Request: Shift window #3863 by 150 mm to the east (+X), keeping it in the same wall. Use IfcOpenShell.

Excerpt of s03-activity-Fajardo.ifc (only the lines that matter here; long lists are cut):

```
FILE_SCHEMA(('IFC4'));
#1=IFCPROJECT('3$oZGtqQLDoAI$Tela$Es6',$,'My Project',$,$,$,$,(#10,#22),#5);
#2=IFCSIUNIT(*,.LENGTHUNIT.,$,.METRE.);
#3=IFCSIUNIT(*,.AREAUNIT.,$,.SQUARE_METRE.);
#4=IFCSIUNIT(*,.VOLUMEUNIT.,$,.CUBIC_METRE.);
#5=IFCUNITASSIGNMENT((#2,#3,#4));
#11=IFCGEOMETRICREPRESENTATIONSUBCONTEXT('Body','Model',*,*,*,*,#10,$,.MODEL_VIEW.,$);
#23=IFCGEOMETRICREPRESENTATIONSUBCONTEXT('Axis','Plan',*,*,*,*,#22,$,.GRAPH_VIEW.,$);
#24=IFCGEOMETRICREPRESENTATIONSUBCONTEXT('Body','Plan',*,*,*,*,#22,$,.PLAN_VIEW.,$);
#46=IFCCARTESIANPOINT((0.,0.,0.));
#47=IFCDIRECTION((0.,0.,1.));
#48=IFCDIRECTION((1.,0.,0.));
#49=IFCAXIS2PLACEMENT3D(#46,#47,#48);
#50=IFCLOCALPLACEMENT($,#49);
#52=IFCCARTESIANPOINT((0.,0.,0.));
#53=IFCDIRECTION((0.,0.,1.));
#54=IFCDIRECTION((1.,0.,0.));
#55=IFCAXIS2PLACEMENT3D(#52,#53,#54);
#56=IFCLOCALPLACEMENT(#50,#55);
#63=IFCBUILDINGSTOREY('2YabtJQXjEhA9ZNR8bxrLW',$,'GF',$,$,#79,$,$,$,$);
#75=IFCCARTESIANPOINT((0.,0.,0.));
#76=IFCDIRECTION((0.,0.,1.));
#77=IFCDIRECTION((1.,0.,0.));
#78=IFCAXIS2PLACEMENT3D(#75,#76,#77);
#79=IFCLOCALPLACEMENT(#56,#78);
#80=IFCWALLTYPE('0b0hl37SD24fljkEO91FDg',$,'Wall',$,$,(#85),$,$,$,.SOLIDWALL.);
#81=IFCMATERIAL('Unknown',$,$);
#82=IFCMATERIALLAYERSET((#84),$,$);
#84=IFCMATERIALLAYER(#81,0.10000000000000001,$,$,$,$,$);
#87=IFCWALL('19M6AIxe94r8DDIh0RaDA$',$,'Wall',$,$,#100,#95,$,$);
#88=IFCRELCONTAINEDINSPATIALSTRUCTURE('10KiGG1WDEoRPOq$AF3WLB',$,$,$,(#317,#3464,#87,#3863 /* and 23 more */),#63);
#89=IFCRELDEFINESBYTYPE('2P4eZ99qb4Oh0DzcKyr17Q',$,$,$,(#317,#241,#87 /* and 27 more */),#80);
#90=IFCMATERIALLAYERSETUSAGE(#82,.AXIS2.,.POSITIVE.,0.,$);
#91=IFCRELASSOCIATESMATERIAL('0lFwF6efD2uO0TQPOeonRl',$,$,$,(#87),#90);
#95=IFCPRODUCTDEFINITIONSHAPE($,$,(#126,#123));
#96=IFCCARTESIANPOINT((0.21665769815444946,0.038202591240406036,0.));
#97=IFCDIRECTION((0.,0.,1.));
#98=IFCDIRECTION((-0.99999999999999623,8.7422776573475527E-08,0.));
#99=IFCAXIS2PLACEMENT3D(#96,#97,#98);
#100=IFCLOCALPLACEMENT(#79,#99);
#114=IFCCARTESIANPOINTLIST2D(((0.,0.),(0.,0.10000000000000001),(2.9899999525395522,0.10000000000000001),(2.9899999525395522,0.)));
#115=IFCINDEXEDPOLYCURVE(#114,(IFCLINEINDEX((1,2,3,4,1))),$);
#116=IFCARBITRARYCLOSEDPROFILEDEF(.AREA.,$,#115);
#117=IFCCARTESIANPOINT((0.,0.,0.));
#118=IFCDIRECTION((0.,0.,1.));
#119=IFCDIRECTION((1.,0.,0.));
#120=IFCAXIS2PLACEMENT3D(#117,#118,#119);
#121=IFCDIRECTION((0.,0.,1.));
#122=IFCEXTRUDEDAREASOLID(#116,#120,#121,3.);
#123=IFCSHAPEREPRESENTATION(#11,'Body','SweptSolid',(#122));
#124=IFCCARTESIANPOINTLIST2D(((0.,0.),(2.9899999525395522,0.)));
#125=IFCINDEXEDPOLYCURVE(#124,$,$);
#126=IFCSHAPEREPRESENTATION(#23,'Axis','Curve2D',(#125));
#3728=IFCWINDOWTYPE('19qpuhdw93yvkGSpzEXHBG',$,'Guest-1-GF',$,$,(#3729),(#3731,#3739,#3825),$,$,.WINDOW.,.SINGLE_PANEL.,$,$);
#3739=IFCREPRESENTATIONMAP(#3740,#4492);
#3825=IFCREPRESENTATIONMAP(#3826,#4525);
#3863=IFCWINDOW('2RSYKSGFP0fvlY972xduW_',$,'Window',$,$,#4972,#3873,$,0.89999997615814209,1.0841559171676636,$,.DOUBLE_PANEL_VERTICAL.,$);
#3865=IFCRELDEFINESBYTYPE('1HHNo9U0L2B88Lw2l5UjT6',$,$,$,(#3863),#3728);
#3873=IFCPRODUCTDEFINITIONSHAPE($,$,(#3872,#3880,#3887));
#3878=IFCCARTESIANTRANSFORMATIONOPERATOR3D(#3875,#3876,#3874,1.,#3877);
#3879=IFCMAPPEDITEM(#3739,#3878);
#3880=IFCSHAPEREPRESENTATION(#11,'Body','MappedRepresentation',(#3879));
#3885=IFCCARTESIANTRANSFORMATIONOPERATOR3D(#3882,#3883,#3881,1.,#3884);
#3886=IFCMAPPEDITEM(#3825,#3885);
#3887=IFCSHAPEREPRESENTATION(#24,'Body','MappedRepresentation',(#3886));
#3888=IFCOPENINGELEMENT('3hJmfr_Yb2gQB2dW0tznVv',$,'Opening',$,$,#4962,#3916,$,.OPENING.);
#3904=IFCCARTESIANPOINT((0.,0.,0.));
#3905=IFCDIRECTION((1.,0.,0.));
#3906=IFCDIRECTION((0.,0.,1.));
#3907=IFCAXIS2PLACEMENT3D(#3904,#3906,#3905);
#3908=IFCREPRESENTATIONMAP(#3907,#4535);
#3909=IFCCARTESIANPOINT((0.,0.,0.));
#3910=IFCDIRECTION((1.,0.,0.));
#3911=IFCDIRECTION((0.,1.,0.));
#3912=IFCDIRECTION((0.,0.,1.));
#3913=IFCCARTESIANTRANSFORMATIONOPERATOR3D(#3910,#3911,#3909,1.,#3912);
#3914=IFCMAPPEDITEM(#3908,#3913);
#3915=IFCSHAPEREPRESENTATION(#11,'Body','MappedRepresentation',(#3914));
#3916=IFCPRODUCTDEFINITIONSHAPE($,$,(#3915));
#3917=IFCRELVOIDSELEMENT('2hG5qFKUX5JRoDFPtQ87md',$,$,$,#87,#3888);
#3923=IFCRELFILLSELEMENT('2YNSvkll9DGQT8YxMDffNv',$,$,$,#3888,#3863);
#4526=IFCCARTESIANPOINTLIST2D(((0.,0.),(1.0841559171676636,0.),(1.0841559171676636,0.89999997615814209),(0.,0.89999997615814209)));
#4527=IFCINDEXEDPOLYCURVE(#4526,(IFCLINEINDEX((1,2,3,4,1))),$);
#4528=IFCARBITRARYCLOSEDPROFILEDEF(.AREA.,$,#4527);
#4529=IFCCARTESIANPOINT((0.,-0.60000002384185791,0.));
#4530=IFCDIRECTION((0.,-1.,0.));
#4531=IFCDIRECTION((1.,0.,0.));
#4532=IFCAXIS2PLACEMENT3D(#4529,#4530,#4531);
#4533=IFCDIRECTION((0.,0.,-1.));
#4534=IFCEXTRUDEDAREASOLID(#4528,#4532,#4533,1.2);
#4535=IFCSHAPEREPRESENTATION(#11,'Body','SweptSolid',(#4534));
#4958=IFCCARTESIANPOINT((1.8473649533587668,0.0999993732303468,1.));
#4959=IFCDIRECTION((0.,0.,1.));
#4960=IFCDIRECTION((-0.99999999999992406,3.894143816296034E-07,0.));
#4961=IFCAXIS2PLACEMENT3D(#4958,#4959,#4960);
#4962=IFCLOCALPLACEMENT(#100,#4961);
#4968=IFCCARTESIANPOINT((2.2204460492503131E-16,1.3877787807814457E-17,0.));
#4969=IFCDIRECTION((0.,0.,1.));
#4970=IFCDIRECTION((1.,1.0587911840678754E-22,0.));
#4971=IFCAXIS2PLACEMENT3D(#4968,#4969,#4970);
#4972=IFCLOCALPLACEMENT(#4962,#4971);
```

```python
import ifcopenshell
import ifcopenshell.api.geometry
import ifcopenshell.util.placement
import ifcopenshell.util.unit

model = ifcopenshell.open("s03-activity-Fajardo.ifc")
unit_scale = ifcopenshell.util.unit.calculate_unit_scale(model)

window = model.by_guid("2RSYKSGFP0fvlY972xduW_")
opening = window.FillsVoids[0].RelatingOpeningElement
wall = opening.VoidsElements[0].RelatingBuildingElement

wall_matrix = ifcopenshell.util.placement.get_local_placement(wall.ObjectPlacement)
shift = wall_matrix[:3, 0] * -0.15 / unit_scale
before = ifcopenshell.util.placement.get_local_placement(window.ObjectPlacement)[:3, 3].copy()

# The window is placed relative to its opening, so it follows when the opening moves.
matrix = ifcopenshell.util.placement.get_local_placement(opening.ObjectPlacement)
matrix[:3, 3] += shift
ifcopenshell.api.geometry.edit_object_placement(
    model, product=opening, matrix=matrix, is_si=False, should_transform_children=True
)

after = ifcopenshell.util.placement.get_local_placement(window.ObjectPlacement)[:3, 3]
print("window moved by", (after - before).round(3) + 0.0)

model.write("s03-activity-Fajardo-out.ifc")
```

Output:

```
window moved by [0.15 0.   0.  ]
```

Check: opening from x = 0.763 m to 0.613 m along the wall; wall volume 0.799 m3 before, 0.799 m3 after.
